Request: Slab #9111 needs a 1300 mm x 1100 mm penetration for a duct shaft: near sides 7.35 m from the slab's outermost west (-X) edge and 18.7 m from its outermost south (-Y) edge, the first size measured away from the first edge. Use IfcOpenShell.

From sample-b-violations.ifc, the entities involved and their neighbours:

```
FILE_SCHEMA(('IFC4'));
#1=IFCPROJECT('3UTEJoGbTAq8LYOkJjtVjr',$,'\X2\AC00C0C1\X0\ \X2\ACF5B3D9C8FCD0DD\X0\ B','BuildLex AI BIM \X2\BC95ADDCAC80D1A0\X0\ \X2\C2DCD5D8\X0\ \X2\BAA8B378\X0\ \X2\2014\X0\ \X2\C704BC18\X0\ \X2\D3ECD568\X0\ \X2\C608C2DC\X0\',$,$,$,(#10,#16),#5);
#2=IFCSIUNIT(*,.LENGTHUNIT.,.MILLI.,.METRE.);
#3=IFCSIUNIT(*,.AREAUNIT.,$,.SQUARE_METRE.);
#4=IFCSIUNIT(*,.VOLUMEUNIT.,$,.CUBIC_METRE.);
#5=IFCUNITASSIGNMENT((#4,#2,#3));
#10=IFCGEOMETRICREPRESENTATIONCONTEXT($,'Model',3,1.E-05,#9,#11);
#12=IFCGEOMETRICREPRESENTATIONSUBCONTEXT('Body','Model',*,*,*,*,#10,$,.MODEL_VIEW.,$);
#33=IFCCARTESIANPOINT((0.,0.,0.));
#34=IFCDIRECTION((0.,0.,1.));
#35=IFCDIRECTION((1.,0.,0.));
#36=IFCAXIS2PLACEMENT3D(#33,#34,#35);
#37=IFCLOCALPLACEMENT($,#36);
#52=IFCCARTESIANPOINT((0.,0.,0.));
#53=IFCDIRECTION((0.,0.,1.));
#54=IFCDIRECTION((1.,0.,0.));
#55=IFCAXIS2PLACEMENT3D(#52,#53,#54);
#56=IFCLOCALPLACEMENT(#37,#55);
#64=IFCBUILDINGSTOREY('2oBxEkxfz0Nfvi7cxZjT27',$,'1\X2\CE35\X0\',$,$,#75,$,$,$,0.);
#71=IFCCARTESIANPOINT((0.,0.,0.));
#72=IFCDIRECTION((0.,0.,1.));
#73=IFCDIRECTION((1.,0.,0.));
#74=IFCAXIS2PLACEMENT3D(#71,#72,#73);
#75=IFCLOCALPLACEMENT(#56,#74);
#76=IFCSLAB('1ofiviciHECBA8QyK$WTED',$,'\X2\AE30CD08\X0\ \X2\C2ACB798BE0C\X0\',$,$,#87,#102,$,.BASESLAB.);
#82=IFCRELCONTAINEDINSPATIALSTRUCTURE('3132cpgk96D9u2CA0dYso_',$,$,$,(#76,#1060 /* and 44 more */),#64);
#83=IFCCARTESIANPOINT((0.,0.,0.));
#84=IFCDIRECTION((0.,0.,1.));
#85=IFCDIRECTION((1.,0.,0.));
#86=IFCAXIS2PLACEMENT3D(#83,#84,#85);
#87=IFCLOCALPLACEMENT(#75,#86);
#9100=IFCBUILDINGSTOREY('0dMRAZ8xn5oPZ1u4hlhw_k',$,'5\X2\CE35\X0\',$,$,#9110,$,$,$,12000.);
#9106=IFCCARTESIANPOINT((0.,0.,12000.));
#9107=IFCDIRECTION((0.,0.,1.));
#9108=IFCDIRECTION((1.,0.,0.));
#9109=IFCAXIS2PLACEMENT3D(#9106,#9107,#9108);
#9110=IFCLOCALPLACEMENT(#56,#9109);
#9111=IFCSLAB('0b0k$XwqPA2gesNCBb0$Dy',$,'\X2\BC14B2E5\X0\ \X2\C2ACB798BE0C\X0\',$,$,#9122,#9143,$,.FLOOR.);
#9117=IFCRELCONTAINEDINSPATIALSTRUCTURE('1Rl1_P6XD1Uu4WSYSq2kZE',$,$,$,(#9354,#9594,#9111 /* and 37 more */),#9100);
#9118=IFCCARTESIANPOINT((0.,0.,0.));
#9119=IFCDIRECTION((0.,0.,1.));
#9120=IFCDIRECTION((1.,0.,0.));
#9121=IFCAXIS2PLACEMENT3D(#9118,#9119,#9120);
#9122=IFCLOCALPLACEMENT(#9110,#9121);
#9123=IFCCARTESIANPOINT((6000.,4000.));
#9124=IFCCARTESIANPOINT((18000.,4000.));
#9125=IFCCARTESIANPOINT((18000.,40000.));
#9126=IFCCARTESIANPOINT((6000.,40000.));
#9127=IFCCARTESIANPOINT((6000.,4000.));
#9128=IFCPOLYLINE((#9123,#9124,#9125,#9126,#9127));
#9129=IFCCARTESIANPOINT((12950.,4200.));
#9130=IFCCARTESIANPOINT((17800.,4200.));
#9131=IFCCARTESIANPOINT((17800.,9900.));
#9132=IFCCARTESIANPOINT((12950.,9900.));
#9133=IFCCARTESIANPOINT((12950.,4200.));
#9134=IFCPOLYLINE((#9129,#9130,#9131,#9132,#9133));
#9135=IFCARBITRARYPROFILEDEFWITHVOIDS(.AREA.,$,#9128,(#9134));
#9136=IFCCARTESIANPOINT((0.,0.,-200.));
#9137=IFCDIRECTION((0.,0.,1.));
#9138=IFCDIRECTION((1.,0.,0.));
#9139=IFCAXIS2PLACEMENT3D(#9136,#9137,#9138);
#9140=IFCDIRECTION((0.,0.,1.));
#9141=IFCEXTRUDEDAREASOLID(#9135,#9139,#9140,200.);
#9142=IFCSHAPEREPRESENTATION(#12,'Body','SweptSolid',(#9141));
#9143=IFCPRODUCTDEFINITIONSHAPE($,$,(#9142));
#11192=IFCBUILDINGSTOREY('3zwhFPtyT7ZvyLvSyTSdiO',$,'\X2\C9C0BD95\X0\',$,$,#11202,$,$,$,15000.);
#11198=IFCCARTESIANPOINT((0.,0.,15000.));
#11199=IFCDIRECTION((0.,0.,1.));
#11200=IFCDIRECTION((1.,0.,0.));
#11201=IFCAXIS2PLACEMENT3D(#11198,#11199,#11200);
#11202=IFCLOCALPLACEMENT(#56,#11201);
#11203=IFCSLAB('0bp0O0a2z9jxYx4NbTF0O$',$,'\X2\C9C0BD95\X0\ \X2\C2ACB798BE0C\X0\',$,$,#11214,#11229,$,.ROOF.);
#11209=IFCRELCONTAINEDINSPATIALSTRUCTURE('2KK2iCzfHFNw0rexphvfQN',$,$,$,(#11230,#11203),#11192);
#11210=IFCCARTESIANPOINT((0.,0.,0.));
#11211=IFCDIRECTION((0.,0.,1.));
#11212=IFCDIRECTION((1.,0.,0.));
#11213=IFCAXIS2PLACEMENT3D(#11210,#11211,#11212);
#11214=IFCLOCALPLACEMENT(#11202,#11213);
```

```python
import numpy as np
import ifcopenshell
import ifcopenshell.api.feature
import ifcopenshell.api.geometry
import ifcopenshell.api.root
import ifcopenshell.geom
import ifcopenshell.util.placement
import ifcopenshell.util.representation
import ifcopenshell.util.shape
import ifcopenshell.util.unit

model = ifcopenshell.open("sample-b-violations.ifc")
unit_scale = ifcopenshell.util.unit.calculate_unit_scale(model)
settings = ifcopenshell.geom.settings()


def volume(element):
    """Net volume in cubic metres, openings subtracted."""
    shape = ifcopenshell.geom.create_shape(settings, element)
    return ifcopenshell.util.shape.get_volume(shape.geometry)


slab = model.by_id(9111)
before = volume(slab)

# Extent in the slab's own axes, in metres. The edges named are its -X and -Y sides.
slab_shape = ifcopenshell.geom.create_shape(settings, slab)
vertices = ifcopenshell.util.shape.get_vertices(slab_shape.geometry)
x_min, y_min, bottom = vertices.min(axis=0)
top = vertices[:, 2].max()

opening = ifcopenshell.api.root.create_entity(model, ifc_class="IfcOpeningElement", name="Duct shaft opening", predefined_type="OPENING")
context = ifcopenshell.util.representation.get_context(model, "Model", "Body", "MODEL_VIEW")
width, depth = 1.3, 1.1
outline = [(0.0, 0.0), (width, 0.0), (width, depth), (0.0, depth), (0.0, 0.0)]
# Overshoot both faces by 50 mm so the cut is clean.
shape = ifcopenshell.api.geometry.add_slab_representation(
    model, context=context, depth=top - bottom + 0.1, polyline=outline
)
ifcopenshell.api.geometry.assign_representation(model, product=opening, representation=shape)

matrix = ifcopenshell.util.placement.get_local_placement(slab.ObjectPlacement)
matrix[:, 3] = matrix @ np.append(np.array([x_min + 7.35, y_min + 18.7, bottom - 0.05]) / unit_scale, 1.0)
ifcopenshell.api.geometry.edit_object_placement(model, product=opening, matrix=matrix, is_si=False)
ifcopenshell.api.feature.add_feature(model, feature=opening, element=slab)

after = volume(slab)

print(f"slab volume {before:.3f} -> {after:.3f} m3")

model.write("sample-b-violations_edited.ifc")
```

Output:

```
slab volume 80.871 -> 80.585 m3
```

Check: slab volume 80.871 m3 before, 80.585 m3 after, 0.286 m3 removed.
